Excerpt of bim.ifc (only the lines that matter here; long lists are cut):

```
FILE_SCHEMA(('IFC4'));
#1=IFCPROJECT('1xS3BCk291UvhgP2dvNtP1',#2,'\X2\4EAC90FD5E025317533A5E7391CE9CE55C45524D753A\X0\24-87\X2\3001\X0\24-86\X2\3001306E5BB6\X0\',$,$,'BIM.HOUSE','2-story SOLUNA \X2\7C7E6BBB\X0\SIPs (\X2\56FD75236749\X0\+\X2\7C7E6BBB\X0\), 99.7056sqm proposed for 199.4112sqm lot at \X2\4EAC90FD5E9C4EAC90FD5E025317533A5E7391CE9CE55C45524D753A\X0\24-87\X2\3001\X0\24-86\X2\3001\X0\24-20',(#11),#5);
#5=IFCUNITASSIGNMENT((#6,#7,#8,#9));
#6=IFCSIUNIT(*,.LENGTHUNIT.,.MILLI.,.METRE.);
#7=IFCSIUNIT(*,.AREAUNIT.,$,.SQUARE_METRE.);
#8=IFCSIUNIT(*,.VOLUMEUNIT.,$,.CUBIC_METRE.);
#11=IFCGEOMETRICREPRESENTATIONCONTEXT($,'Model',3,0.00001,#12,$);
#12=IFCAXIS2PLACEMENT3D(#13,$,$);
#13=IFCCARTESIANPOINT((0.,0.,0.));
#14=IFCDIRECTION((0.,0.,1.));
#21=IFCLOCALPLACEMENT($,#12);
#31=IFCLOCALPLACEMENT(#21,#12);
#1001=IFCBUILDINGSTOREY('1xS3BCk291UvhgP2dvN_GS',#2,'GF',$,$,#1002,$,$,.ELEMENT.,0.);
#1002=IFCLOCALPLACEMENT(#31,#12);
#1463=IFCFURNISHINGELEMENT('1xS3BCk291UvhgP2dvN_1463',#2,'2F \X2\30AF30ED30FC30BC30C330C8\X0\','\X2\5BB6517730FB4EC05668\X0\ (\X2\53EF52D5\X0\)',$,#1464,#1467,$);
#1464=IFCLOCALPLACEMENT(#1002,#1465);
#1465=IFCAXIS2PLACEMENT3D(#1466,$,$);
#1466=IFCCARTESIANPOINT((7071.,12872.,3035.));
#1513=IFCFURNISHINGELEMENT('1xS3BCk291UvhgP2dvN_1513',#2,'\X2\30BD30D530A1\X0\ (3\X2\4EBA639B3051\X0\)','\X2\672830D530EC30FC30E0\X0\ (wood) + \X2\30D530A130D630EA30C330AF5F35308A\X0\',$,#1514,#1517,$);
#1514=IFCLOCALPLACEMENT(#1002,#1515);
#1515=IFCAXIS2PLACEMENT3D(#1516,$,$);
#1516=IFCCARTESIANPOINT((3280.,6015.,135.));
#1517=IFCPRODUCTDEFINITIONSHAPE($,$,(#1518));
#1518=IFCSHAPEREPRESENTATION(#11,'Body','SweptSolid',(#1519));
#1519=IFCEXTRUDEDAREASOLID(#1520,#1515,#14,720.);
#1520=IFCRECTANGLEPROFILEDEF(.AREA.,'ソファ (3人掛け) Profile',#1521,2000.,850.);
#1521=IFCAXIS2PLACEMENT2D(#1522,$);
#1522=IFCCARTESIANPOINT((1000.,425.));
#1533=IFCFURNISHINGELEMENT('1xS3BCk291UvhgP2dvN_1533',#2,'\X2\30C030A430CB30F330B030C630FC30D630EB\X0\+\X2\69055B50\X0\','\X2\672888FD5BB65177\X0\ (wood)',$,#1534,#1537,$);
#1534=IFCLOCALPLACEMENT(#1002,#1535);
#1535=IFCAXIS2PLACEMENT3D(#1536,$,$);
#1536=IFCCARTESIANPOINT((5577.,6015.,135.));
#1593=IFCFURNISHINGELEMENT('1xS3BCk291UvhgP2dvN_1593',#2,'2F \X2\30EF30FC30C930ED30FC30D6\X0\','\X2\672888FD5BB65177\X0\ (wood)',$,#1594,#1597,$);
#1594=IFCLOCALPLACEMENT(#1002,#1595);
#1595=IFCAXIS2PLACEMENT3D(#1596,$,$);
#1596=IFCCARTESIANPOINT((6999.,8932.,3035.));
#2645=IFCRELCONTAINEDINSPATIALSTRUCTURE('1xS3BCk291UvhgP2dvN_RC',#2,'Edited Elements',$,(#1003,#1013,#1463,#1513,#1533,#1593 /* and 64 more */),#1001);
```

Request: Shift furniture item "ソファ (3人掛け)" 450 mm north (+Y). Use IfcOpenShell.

```python
import ifcopenshell
import ifcopenshell.api.geometry
import ifcopenshell.util.placement
import ifcopenshell.util.unit

model = ifcopenshell.open("bim.ifc")
unit_scale = ifcopenshell.util.unit.calculate_unit_scale(model)

item = model.by_guid("1xS3BCk291UvhgP2dvN_1513")
matrix = ifcopenshell.util.placement.get_local_placement(item.ObjectPlacement)
matrix[1, 3] += 0.45 / unit_scale
ifcopenshell.api.geometry.edit_object_placement(model, product=item, matrix=matrix, is_si=False)

print(ifcopenshell.util.placement.get_local_placement(item.ObjectPlacement).round(3) + 0.0)

model.write("bim_rev.ifc")
```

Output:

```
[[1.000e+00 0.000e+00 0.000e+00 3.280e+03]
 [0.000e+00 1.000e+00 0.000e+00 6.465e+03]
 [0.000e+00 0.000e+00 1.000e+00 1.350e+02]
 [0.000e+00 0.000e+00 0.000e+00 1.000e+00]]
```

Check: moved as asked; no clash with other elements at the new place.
